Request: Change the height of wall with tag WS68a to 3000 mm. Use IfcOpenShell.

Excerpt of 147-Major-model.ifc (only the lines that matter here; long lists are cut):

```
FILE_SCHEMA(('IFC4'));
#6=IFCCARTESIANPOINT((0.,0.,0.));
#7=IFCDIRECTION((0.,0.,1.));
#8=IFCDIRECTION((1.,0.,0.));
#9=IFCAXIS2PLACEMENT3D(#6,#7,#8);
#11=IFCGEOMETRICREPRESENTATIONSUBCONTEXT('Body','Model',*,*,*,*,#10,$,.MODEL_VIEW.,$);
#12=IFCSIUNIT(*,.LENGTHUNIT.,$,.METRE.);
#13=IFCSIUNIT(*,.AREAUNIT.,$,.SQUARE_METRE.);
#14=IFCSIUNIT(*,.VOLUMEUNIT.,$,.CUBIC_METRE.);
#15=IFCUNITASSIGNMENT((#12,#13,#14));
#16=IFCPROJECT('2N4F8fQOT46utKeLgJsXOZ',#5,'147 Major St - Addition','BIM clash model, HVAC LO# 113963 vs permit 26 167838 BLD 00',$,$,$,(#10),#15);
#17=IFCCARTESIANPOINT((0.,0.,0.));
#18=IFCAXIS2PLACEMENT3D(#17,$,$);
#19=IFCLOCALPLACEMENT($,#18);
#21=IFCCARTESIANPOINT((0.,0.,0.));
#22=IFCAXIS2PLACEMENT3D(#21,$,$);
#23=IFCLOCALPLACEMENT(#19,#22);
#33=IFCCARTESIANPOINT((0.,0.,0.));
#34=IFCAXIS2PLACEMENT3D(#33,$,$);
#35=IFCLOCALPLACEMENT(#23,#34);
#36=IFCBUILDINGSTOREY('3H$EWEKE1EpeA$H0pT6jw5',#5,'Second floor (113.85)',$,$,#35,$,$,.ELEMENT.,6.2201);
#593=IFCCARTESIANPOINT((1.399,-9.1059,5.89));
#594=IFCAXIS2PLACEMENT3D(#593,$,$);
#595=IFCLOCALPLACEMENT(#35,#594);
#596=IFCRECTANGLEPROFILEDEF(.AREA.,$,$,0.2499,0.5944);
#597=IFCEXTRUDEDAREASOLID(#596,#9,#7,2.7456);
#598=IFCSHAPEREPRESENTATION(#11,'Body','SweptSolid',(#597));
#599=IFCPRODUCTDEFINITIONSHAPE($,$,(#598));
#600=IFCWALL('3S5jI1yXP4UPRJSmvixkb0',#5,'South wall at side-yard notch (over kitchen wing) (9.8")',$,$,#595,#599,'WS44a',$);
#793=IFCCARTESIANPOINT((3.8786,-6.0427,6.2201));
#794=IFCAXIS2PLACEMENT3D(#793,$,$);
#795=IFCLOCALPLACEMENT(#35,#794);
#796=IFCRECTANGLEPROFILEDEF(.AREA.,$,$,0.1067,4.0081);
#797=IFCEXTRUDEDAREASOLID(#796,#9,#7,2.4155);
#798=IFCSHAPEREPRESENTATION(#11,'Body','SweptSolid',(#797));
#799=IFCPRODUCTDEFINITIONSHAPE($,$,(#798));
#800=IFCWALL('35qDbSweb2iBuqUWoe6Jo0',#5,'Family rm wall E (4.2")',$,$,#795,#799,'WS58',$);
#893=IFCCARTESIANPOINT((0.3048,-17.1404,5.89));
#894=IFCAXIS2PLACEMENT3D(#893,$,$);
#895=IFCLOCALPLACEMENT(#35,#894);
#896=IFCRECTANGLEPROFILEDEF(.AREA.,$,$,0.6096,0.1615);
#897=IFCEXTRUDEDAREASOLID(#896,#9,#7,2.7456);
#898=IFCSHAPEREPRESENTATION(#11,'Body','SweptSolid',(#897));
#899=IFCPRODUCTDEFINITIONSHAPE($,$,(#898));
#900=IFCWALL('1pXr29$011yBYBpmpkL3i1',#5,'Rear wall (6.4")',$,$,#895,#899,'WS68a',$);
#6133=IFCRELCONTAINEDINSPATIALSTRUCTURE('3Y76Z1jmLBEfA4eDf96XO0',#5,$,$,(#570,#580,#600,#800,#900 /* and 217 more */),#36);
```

```python
import ifcopenshell
import ifcopenshell.geom
import ifcopenshell.util.representation
import ifcopenshell.util.shape
import ifcopenshell.util.unit

model = ifcopenshell.open("147-Major-model.ifc")
unit_scale = ifcopenshell.util.unit.calculate_unit_scale(model)
settings = ifcopenshell.geom.settings()


def volume(element):
    """Net volume in cubic metres, openings subtracted."""
    shape = ifcopenshell.geom.create_shape(settings, element)
    return ifcopenshell.util.shape.get_volume(shape.geometry)


wall = model.by_guid("1pXr29$011yBYBpmpkL3i1")
before = volume(wall)

body = ifcopenshell.util.representation.get_representation(wall, "Model", "Body")
solid = body.Items[0]
old_height = solid.Depth
solid.Depth = 3 / unit_scale
after = volume(wall)

print(f"height {old_height:g} -> {solid.Depth:g}, volume {before:.3f} -> {after:.3f} m3")

model.write("147-Major-model_edited.ifc")
```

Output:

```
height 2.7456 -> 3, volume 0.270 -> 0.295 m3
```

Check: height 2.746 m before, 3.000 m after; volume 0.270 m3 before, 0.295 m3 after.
